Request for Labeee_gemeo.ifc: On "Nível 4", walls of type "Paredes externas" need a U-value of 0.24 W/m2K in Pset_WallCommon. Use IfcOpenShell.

First a look at what the model holds.

```python
import ifcopenshell
import ifcopenshell.util.element

model = ifcopenshell.open("Labeee_gemeo.ifc")
print(model.schema)
storey = next(s for s in model.by_type("IfcBuildingStorey") if s.Name == "Nível 4")
walls = [e for e in ifcopenshell.util.element.get_decomposition(storey) if e.is_a("IfcWall")]
seen = {}
for e in walls:
    element_type = ifcopenshell.util.element.get_type(e)
    key = (element_type.Name if element_type != e and element_type else None, ifcopenshell.util.element.get_pset(e, "Pset_WallCommon", "ThermalTransmittance"))
    seen[key] = seen.get(key, 0) + 1
for (name, value), count in sorted(seen.items(), key=str):
    print(count, "x", name, "|", value)
```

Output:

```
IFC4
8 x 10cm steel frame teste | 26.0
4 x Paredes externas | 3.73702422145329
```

```python
import ifcopenshell
import ifcopenshell.api.pset
import ifcopenshell.util.element

model = ifcopenshell.open("Labeee_gemeo.ifc")

storey = next(s for s in model.by_type("IfcBuildingStorey") if s.Name == "Nível 4")
walls = [e for e in ifcopenshell.util.element.get_decomposition(storey) if e.is_a("IfcWall")]

count = 0
for e in walls:
    element_type = ifcopenshell.util.element.get_type(e)
    if element_type in (None, e) or element_type.Name != "Paredes externas":
        continue
    # add_pset returns the element's existing set when there is one.
    pset = ifcopenshell.api.pset.add_pset(model, product=e, name="Pset_WallCommon")
    ifcopenshell.api.pset.edit_pset(model, pset=pset, properties={"ThermalTransmittance": 0.24})
    count += 1

print(count, "walls updated")

model.write("Labeee_gemeo-out.ifc")
```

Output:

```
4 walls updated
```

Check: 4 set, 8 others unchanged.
